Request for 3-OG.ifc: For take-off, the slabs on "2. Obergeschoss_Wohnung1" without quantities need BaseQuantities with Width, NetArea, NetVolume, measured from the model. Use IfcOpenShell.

First a look at what the model holds.

```python
import ifcopenshell
import ifcopenshell.util.element
import ifcopenshell.util.unit

model = ifcopenshell.open("3-OG.ifc")
print(model.schema)
for unit_type in ("LENGTHUNIT", "AREAUNIT", "VOLUMEUNIT"):
    print(unit_type, ifcopenshell.util.unit.calculate_unit_scale(model, unit_type))
storey = next(s for s in model.by_type("IfcBuildingStorey") if s.Name == "2. Obergeschoss_Wohnung1")
slabs = [e for e in ifcopenshell.util.element.get_decomposition(storey) if e.is_a("IfcSlab")]
for e in sorted(slabs, key=lambda e: e.id()):
    print(e.id(), e.is_a(), e.Name, list(ifcopenshell.util.element.get_psets(e, qtos_only=True)), sep=" | ")
```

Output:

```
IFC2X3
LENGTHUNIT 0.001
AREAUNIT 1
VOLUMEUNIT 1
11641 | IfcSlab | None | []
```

```python
import ifcopenshell
import ifcopenshell.api.pset
import ifcopenshell.geom
import ifcopenshell.util.element
import ifcopenshell.util.shape
import ifcopenshell.util.unit

model = ifcopenshell.open("3-OG.ifc")
unit_scale = ifcopenshell.util.unit.calculate_unit_scale(model)
area_scale = ifcopenshell.util.unit.calculate_unit_scale(model, "AREAUNIT")
volume_scale = ifcopenshell.util.unit.calculate_unit_scale(model, "VOLUMEUNIT")
settings = ifcopenshell.geom.settings()

storey = next(s for s in model.by_type("IfcBuildingStorey") if s.Name == "2. Obergeschoss_Wohnung1")
slabs = [e for e in ifcopenshell.util.element.get_decomposition(storey) if e.is_a("IfcSlab")]

for e in sorted(slabs, key=lambda e: e.id()):
    if ifcopenshell.util.element.get_psets(e, qtos_only=True, should_inherit=False):
        continue
    # Geometry comes back in metres, in the element's own axes.
    shape = ifcopenshell.geom.create_shape(settings, e)
    values = {
        "Width": ifcopenshell.util.shape.get_z(shape.geometry) / unit_scale,
        "NetArea": ifcopenshell.util.shape.get_footprint_area(shape.geometry) / area_scale,
        "NetVolume": ifcopenshell.util.shape.get_volume(shape.geometry) / volume_scale,
    }
    qto = ifcopenshell.api.pset.add_qto(model, product=e, name="BaseQuantities")
    ifcopenshell.api.pset.edit_qto(model, qto=qto, properties=values)
    print(e.id(), {k: round(v, 3) for k, v in values.items()})

model.write("3-OG_updated.ifc")
```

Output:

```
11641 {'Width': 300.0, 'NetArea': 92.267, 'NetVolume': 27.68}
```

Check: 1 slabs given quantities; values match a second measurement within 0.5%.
